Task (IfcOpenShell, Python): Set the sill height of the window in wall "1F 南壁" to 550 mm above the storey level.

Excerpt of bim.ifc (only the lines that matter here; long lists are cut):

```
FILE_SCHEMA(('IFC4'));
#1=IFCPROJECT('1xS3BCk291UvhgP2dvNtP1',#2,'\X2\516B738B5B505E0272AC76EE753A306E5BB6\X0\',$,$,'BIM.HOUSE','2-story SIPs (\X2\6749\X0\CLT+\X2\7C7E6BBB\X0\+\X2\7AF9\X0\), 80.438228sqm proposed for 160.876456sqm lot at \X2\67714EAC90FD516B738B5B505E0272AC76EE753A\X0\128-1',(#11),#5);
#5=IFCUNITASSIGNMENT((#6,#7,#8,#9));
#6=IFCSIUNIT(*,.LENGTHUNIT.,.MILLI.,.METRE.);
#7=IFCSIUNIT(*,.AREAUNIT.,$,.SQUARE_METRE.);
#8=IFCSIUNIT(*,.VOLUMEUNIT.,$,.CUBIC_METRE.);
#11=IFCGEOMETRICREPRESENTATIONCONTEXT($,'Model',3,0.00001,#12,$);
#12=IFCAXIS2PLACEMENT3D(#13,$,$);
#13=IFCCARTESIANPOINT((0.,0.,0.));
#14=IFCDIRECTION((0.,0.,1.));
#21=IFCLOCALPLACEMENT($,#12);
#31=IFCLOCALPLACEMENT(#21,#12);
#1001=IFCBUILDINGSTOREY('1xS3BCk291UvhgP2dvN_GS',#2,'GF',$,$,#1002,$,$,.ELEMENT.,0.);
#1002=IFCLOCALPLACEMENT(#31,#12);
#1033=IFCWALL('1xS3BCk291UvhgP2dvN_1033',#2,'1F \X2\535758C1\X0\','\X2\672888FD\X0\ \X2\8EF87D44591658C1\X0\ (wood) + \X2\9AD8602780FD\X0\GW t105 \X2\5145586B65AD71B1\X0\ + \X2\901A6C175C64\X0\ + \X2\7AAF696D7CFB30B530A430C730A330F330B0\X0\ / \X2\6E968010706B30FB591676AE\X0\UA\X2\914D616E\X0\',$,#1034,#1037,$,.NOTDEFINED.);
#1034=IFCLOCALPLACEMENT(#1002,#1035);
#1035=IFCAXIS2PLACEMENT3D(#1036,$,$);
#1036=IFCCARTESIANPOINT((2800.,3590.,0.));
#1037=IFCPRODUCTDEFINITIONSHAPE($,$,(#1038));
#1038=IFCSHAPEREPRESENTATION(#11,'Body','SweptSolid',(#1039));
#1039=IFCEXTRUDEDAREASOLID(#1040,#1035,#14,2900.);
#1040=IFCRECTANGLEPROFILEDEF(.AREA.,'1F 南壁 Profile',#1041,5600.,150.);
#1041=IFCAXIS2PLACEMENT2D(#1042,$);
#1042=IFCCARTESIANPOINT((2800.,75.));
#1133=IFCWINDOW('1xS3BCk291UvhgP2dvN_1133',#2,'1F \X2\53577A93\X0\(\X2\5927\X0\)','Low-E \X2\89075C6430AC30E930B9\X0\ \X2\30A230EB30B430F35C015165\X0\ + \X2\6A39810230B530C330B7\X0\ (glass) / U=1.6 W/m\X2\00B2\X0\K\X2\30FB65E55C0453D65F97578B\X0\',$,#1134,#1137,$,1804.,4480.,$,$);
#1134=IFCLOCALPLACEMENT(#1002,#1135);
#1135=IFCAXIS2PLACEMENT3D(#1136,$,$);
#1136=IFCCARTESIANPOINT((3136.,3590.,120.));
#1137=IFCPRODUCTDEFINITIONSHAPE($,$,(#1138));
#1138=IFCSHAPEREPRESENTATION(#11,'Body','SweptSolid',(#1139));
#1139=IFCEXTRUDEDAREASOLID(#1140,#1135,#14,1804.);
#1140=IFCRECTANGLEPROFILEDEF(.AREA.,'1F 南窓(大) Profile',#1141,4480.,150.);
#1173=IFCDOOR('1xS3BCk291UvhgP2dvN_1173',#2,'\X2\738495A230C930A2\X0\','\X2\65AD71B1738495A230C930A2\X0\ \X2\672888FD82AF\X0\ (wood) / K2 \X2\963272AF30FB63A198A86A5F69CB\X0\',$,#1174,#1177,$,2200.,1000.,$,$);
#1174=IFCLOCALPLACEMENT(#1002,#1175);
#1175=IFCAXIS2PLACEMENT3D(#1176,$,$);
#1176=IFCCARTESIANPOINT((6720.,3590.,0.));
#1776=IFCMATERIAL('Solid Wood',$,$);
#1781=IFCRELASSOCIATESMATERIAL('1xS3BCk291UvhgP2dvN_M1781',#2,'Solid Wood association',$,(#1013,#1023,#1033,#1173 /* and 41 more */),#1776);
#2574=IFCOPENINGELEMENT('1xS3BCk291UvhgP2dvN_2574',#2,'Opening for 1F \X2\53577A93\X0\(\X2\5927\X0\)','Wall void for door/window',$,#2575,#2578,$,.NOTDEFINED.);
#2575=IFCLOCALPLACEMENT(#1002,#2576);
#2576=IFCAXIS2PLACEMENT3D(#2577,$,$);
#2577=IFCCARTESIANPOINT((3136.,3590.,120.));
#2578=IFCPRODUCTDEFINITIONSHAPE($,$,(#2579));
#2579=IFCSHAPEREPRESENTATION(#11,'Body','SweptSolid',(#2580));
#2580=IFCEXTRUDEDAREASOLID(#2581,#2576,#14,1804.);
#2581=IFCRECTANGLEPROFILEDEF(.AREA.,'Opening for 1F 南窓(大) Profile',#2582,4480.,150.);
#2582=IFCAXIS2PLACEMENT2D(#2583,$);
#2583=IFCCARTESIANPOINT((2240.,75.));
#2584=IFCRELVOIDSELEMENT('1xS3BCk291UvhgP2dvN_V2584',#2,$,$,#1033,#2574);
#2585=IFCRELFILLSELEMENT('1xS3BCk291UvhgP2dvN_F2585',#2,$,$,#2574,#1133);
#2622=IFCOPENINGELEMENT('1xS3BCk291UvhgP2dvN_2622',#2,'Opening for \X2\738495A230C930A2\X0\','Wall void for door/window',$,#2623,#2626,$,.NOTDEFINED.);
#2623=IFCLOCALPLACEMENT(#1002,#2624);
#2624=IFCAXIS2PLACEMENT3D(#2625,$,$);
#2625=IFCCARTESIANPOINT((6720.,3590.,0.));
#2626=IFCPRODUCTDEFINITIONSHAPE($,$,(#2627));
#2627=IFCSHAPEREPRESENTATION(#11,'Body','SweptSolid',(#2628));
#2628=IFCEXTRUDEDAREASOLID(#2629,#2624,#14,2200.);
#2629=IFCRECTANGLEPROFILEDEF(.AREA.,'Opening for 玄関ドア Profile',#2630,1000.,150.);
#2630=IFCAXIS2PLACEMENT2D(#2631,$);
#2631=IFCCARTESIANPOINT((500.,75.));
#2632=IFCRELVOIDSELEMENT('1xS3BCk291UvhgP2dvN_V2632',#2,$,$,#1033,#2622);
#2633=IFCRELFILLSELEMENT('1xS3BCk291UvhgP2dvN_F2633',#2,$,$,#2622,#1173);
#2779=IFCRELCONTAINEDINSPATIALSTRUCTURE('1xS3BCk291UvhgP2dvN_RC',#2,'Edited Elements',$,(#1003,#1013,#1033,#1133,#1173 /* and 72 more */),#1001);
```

```python
import numpy as np
import ifcopenshell
import ifcopenshell.api.geometry
import ifcopenshell.geom
import ifcopenshell.util.element
import ifcopenshell.util.placement
import ifcopenshell.util.shape
import ifcopenshell.util.unit

model = ifcopenshell.open("bim.ifc")
unit_scale = ifcopenshell.util.unit.calculate_unit_scale(model)

window = model.by_id(1133)
opening = window.FillsVoids[0].RelatingOpeningElement
storey = ifcopenshell.util.element.get_container(window, ifc_class="IfcBuildingStorey")
level = ifcopenshell.util.placement.get_local_placement(storey.ObjectPlacement)[2, 3]

# The opening's origin need not be at the sill, so measure its lowest point.
shape = ifcopenshell.geom.create_shape(ifcopenshell.geom.settings(), opening)
bottom = ifcopenshell.util.shape.get_shape_bottom_elevation(shape, shape.geometry) / unit_scale
dz = level + 0.55 / unit_scale - bottom

shift = np.array([0.0, 0.0, dz])
# The window is not placed relative to its opening, so move both.
for product in (opening, window):
    matrix = ifcopenshell.util.placement.get_local_placement(product.ObjectPlacement)
    matrix[:3, 3] += shift
    ifcopenshell.api.geometry.edit_object_placement(model, product=product, matrix=matrix, is_si=False)

print(f"moved by {dz * unit_scale:+.3f} m")

model.write("bim_rev.ifc")
```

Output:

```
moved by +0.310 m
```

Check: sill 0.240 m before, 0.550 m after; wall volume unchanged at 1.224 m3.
